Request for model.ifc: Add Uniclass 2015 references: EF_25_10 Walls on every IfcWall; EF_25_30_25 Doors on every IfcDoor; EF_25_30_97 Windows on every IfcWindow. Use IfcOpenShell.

First a look at what the model holds.

```python
import ifcopenshell

model = ifcopenshell.open("model.ifc")
print(model.schema)
print("classifications:", [c.Name for c in model.by_type("IfcClassification")])
for ifc_class in ("IfcDoor", "IfcRoof", "IfcStair", "IfcWall", "IfcWindow"):
    print(ifc_class, len(model.by_type(ifc_class)))
```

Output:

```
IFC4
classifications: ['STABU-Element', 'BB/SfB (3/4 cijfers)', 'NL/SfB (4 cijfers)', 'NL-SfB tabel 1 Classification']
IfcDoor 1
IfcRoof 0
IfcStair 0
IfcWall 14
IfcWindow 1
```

```python
import ifcopenshell
import ifcopenshell.api.classification

model = ifcopenshell.open("model.ifc")

system = ifcopenshell.api.classification.add_classification(model, classification="Uniclass 2015")

codes = {
    "IfcWall": ("EF_25_10", "Walls"),
    "IfcDoor": ("EF_25_30_25", "Doors"),
    "IfcWindow": ("EF_25_30_97", "Windows"),
}
for ifc_class, (code, name) in codes.items():
    products = model.by_type(ifc_class)
    ifcopenshell.api.classification.add_reference(
        model, products=products, classification=system, identification=code, name=name
    )
    print(code, len(products))

model.write("model_updated.ifc")
```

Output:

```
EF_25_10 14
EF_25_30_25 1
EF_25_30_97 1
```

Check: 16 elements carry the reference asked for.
